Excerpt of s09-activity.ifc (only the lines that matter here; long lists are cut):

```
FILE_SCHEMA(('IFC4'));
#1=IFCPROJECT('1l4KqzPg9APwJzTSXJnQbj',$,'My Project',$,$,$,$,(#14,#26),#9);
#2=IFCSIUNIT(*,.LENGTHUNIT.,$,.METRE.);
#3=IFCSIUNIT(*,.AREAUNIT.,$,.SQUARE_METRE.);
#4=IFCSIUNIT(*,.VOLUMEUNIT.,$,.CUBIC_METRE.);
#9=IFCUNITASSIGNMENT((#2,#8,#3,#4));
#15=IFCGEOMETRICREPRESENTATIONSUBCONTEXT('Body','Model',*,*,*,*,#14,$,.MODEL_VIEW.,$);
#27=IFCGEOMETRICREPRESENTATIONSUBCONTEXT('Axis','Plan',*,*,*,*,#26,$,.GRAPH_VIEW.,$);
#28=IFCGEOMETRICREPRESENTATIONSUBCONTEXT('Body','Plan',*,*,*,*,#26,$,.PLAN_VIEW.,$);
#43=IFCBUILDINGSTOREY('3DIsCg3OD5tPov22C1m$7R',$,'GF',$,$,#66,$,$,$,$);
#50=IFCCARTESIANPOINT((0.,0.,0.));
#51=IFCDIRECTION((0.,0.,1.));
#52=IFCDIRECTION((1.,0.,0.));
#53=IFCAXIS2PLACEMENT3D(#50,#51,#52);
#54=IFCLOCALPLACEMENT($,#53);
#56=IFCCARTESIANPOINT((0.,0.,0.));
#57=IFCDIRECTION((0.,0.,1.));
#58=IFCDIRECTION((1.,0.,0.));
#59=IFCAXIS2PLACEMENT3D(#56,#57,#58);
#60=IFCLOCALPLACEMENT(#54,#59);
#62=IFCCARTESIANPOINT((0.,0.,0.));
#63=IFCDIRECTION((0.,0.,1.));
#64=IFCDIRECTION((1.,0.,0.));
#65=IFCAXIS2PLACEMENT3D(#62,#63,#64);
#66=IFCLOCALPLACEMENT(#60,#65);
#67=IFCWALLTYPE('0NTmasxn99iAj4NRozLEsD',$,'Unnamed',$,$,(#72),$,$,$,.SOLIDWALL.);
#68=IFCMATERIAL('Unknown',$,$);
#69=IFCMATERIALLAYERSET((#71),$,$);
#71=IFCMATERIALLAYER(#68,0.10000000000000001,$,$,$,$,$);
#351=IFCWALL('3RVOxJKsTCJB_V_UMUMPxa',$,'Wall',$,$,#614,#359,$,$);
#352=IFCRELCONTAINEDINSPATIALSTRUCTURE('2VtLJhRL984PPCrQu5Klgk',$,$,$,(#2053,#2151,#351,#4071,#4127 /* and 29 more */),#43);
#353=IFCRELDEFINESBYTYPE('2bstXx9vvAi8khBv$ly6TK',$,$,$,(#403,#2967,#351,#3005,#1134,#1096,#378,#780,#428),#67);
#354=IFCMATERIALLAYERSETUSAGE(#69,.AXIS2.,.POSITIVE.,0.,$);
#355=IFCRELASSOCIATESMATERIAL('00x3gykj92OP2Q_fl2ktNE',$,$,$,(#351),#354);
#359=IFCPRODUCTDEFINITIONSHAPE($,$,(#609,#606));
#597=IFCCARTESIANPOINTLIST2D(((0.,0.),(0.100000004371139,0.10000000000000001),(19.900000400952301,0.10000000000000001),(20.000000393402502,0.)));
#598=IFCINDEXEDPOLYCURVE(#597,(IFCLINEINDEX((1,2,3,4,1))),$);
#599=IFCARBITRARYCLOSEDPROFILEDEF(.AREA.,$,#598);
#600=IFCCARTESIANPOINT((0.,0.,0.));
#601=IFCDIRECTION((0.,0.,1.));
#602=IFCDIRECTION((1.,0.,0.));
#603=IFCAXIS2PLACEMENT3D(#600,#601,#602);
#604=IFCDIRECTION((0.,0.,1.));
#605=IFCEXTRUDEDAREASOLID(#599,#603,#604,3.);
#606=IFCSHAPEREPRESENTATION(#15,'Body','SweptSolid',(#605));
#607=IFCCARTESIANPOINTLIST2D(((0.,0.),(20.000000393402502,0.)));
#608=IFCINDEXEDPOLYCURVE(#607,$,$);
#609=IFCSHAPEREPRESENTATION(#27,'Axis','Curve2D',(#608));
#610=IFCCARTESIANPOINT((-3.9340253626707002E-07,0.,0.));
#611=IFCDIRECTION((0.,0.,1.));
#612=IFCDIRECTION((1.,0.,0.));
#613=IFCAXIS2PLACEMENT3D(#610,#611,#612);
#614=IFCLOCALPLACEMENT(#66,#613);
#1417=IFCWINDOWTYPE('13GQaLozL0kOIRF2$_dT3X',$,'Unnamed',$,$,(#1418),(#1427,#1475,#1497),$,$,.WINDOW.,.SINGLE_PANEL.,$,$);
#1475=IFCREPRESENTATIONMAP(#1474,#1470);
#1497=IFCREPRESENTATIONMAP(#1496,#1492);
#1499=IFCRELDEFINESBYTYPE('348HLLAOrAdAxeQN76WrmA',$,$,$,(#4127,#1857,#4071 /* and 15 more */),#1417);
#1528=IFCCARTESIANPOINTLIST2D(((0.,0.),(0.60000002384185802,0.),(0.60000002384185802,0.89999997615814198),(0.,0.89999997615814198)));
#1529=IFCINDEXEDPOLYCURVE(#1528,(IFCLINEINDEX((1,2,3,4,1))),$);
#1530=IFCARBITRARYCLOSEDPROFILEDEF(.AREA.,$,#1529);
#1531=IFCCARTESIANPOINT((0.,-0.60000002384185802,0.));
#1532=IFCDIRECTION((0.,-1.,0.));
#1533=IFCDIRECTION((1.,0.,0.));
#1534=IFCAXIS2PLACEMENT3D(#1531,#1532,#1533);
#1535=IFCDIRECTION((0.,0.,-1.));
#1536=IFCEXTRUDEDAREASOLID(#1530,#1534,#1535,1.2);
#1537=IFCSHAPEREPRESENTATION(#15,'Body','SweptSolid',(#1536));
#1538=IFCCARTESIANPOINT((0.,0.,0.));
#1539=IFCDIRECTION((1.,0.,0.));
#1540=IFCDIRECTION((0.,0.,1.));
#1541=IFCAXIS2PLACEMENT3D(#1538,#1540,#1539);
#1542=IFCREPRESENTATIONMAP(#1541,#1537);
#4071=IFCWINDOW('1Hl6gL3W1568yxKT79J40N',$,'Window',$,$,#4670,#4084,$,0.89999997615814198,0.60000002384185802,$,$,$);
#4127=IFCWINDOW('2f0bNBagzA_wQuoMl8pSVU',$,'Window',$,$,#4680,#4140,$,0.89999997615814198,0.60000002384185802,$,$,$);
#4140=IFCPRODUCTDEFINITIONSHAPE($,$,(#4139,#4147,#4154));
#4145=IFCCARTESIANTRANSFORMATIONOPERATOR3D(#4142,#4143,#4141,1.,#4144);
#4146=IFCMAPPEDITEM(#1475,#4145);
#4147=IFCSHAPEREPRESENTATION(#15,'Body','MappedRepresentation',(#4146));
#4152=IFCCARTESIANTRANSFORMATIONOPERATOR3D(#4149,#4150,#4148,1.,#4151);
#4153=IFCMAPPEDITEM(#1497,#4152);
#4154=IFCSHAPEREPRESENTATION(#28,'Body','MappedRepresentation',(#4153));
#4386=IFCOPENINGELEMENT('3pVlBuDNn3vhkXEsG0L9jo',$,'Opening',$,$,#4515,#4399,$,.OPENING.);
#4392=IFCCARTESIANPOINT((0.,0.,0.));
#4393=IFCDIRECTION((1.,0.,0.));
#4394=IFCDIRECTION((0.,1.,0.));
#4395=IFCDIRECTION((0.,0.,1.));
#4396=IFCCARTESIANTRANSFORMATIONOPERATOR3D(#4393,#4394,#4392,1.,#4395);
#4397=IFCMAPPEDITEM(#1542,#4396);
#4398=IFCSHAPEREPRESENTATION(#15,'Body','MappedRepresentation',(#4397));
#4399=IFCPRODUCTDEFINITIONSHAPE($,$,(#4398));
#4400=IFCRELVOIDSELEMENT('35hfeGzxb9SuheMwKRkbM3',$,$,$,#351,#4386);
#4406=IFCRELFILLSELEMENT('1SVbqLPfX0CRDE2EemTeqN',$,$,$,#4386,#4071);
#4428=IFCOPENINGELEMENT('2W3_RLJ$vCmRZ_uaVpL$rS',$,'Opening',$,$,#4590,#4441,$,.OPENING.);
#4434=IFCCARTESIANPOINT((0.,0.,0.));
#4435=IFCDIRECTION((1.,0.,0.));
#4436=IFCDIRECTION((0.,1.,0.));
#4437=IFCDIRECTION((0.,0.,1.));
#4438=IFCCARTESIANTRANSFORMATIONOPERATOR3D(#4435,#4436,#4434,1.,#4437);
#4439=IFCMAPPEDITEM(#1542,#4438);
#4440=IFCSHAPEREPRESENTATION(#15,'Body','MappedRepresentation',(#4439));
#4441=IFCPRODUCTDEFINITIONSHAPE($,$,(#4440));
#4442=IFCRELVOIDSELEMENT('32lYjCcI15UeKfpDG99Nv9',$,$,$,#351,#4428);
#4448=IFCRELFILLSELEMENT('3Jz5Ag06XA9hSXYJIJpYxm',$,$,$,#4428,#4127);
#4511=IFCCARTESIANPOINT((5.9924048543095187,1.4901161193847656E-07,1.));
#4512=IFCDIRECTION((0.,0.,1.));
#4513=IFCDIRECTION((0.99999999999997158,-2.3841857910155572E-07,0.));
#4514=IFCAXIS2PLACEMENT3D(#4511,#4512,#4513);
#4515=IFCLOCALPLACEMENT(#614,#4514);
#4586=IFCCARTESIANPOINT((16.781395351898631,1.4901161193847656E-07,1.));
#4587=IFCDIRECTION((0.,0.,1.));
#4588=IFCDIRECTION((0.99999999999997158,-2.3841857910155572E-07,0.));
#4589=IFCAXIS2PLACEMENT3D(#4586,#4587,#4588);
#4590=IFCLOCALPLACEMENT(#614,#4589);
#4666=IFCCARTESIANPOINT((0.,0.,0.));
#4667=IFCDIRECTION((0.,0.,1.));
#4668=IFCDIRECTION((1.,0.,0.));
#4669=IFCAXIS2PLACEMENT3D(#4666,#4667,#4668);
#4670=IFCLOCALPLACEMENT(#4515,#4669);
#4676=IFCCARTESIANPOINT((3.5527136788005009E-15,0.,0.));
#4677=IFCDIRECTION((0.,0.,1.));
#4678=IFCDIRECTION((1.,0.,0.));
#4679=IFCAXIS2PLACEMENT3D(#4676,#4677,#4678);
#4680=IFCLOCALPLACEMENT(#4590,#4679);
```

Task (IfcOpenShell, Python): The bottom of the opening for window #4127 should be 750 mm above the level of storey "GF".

```python
import numpy as np
import ifcopenshell
import ifcopenshell.api.geometry
import ifcopenshell.geom
import ifcopenshell.util.element
import ifcopenshell.util.placement
import ifcopenshell.util.shape
import ifcopenshell.util.unit

model = ifcopenshell.open("s09-activity.ifc")
unit_scale = ifcopenshell.util.unit.calculate_unit_scale(model)

window = model.by_guid("2f0bNBagzA_wQuoMl8pSVU")
opening = window.FillsVoids[0].RelatingOpeningElement
storey = ifcopenshell.util.element.get_container(window, ifc_class="IfcBuildingStorey")
level = ifcopenshell.util.placement.get_local_placement(storey.ObjectPlacement)[2, 3]

# The opening's origin need not be at the sill, so measure its lowest point.
shape = ifcopenshell.geom.create_shape(ifcopenshell.geom.settings(), opening)
bottom = ifcopenshell.util.shape.get_shape_bottom_elevation(shape, shape.geometry) / unit_scale
dz = level + 0.75 - bottom

shift = np.array([0.0, 0.0, dz])
# The window is placed relative to its opening, so it follows when the opening moves.
matrix = ifcopenshell.util.placement.get_local_placement(opening.ObjectPlacement)
matrix[:3, 3] += shift
ifcopenshell.api.geometry.edit_object_placement(
    model, product=opening, matrix=matrix, is_si=False, should_transform_children=True
)

print(f"moved by {dz * unit_scale:+.3f} m")

model.write("s09-activity-out.ifc")
```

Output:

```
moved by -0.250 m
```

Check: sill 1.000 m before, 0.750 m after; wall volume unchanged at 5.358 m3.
